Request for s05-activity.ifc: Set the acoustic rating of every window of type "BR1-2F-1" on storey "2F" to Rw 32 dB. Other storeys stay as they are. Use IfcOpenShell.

First a look at what the model holds.

```python
import ifcopenshell
import ifcopenshell.util.element

model = ifcopenshell.open("s05-activity.ifc")
print(model.schema)
storey = next(s for s in model.by_type("IfcBuildingStorey") if s.Name == "2F")
windows = [e for e in ifcopenshell.util.element.get_decomposition(storey) if e.is_a("IfcWindow")]
seen = {}
for e in windows:
    element_type = ifcopenshell.util.element.get_type(e)
    key = (element_type.Name if element_type != e and element_type else None, ifcopenshell.util.element.get_pset(e, "Pset_WindowCommon", "AcousticRating"))
    seen[key] = seen.get(key, 0) + 1
for (name, value), count in sorted(seen.items(), key=str):
    print(count, "x", name, "|", value)
```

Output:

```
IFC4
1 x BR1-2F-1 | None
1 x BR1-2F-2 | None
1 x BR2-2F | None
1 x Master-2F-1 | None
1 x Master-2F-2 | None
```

```python
import ifcopenshell
import ifcopenshell.api.pset
import ifcopenshell.util.element

model = ifcopenshell.open("s05-activity.ifc")

storey = next(s for s in model.by_type("IfcBuildingStorey") if s.Name == "2F")
windows = [e for e in ifcopenshell.util.element.get_decomposition(storey) if e.is_a("IfcWindow")]

count = 0
for e in windows:
    element_type = ifcopenshell.util.element.get_type(e)
    if element_type in (None, e) or element_type.Name != "BR1-2F-1":
        continue
    # add_pset returns the element's existing set when there is one.
    pset = ifcopenshell.api.pset.add_pset(model, product=e, name="Pset_WindowCommon")
    ifcopenshell.api.pset.edit_pset(model, pset=pset, properties={"AcousticRating": "Rw 32 dB"})
    count += 1

print(count, "windows updated")

model.write("s05-activity_v2.ifc")
```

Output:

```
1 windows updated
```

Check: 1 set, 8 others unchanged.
